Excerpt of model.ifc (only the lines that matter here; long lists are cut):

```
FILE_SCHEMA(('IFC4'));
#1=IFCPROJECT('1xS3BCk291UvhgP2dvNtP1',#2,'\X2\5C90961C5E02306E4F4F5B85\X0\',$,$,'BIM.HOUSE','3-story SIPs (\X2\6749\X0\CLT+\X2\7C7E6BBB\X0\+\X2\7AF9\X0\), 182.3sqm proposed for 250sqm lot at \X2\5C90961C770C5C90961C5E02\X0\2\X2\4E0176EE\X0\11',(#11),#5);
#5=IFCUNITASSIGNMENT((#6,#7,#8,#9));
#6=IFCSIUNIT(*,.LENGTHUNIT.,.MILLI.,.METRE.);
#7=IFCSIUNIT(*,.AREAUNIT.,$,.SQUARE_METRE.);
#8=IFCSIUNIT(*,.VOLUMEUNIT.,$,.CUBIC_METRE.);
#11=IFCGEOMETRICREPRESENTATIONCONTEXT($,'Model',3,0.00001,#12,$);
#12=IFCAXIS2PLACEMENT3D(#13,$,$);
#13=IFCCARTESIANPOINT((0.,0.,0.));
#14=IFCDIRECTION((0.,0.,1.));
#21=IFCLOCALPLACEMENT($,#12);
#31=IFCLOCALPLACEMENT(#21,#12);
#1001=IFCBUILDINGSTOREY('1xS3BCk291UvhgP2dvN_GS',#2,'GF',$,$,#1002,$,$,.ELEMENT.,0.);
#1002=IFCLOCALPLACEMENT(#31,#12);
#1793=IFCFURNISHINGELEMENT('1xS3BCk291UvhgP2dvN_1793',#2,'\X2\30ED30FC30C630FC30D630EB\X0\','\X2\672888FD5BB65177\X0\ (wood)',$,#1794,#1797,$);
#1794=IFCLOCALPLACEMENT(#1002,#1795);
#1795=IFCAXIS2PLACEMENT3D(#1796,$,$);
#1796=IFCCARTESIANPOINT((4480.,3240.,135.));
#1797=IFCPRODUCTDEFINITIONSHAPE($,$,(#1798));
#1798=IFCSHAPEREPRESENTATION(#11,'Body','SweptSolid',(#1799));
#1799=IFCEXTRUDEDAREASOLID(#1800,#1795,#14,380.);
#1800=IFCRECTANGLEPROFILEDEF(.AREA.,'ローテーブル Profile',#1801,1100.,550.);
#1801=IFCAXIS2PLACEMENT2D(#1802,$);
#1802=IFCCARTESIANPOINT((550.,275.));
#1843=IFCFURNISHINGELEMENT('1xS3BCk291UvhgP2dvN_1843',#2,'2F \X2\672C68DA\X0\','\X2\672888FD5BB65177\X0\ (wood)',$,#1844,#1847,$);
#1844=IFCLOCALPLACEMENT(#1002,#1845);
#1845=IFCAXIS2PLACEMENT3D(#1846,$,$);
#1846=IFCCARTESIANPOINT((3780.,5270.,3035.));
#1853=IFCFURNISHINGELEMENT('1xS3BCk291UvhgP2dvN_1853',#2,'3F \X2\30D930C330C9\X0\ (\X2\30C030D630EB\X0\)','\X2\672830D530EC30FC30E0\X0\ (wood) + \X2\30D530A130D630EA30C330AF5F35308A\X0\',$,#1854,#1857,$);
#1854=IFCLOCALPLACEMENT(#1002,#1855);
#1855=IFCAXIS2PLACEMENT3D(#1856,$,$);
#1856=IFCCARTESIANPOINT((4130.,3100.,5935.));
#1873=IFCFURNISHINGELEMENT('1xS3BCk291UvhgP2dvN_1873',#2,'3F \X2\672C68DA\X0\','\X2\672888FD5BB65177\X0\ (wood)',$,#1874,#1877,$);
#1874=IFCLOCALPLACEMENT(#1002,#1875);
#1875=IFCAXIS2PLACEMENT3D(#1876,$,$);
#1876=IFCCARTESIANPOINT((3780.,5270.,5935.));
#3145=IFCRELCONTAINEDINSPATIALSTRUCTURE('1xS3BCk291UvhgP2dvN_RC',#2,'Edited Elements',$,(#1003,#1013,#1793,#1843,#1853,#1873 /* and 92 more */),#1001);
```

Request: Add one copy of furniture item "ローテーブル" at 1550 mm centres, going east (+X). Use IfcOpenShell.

```python
import numpy as np
import ifcopenshell
import ifcopenshell.api.geometry
import ifcopenshell.api.root
import ifcopenshell.util.element
import ifcopenshell.util.placement

model = ifcopenshell.open("model.ifc")


def reuse_history(source, copy):
    """copy_class also copies each property set's owner history, people and application; keep the originals."""
    for rel in copy.IsDefinedBy:
        if rel.is_a("IfcRelDefinesByProperties") and (history := rel.RelatingPropertyDefinition.OwnerHistory):
            rel.RelatingPropertyDefinition.OwnerHistory = source.OwnerHistory
            ifcopenshell.util.element.remove_deep2(model, history)


source = model.by_guid("1xS3BCk291UvhgP2dvN_1793")
base = ifcopenshell.util.placement.get_local_placement(source.ObjectPlacement)
step = np.array([1.0, 0.0, 0.0]) * 1550.0

for i in range(1, 2):
    copy = ifcopenshell.api.root.copy_class(model, product=source)
    copy.Representation = ifcopenshell.util.element.copy_deep(
        model, source.Representation, exclude=["IfcGeometricRepresentationContext", "IfcRepresentationMap"]
    )
    reuse_history(source, copy)
    matrix = base.copy()
    matrix[:3, 3] += i * step
    print("added at", matrix[:3, 3].round(3) + 0.0)
    ifcopenshell.api.geometry.edit_object_placement(model, product=copy, matrix=matrix, is_si=False)

model.write("model-out.ifc")
```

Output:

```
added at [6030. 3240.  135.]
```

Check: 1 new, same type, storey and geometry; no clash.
